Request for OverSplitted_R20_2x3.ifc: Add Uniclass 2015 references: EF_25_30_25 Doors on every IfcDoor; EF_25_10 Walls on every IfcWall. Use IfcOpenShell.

First a look at what the model holds.

```python
import ifcopenshell

model = ifcopenshell.open("OverSplitted_R20_2x3.ifc")
print(model.schema)
print("classifications:", [c.Name for c in model.by_type("IfcClassification")])
for ifc_class in ("IfcDoor", "IfcRoof", "IfcStair", "IfcWall", "IfcWindow"):
    print(ifc_class, len(model.by_type(ifc_class)))
```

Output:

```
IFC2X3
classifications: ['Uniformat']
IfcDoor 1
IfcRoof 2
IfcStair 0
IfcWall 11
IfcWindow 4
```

```python
import ifcopenshell
import ifcopenshell.api.classification

model = ifcopenshell.open("OverSplitted_R20_2x3.ifc")

# IFC2X3 requires Source and Edition and has no link from the project to the system.
system = model.create_entity("IfcClassification", Source="NBS", Edition="2015", Name="Uniclass 2015")

codes = {
    "IfcDoor": ("EF_25_30_25", "Doors"),
    "IfcWall": ("EF_25_10", "Walls"),
}
for ifc_class, (code, name) in codes.items():
    products = model.by_type(ifc_class)
    ifcopenshell.api.classification.add_reference(
        model, products=products, classification=system, identification=code, name=name
    )
    print(code, len(products))

model.write("OverSplitted_R20_2x3_updated.ifc")
```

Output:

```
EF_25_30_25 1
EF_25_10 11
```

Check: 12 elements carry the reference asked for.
